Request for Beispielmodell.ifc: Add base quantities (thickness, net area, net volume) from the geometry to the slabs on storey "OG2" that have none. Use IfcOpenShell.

First a look at what the model holds.

```python
import ifcopenshell
import ifcopenshell.util.element
import ifcopenshell.util.unit

model = ifcopenshell.open("Beispielmodell.ifc")
print(model.schema)
for unit_type in ("LENGTHUNIT", "AREAUNIT", "VOLUMEUNIT"):
    print(unit_type, ifcopenshell.util.unit.calculate_unit_scale(model, unit_type))
storey = next(s for s in model.by_type("IfcBuildingStorey") if s.Name == "OG2")
slabs = [e for e in ifcopenshell.util.element.get_decomposition(storey) if e.is_a("IfcSlab")]
for e in sorted(slabs, key=lambda e: e.id()):
    print(e.id(), e.is_a(), e.Name, list(ifcopenshell.util.element.get_psets(e, qtos_only=True)), sep=" | ")
```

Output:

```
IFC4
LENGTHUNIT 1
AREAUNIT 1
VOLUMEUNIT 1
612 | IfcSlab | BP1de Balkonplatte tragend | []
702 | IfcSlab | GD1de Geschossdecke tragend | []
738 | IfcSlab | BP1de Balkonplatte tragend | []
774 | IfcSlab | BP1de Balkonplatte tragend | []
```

```python
import ifcopenshell
import ifcopenshell.api.pset
import ifcopenshell.geom
import ifcopenshell.util.element
import ifcopenshell.util.shape
import ifcopenshell.util.unit

model = ifcopenshell.open("Beispielmodell.ifc")
unit_scale = ifcopenshell.util.unit.calculate_unit_scale(model)
area_scale = ifcopenshell.util.unit.calculate_unit_scale(model, "AREAUNIT")
volume_scale = ifcopenshell.util.unit.calculate_unit_scale(model, "VOLUMEUNIT")
settings = ifcopenshell.geom.settings()

storey = next(s for s in model.by_type("IfcBuildingStorey") if s.Name == "OG2")
slabs = [e for e in ifcopenshell.util.element.get_decomposition(storey) if e.is_a("IfcSlab")]

for e in sorted(slabs, key=lambda e: e.id()):
    if ifcopenshell.util.element.get_psets(e, qtos_only=True, should_inherit=False):
        continue
    # Geometry comes back in metres, in the element's own axes.
    shape = ifcopenshell.geom.create_shape(settings, e)
    values = {
        "Width": ifcopenshell.util.shape.get_z(shape.geometry) / unit_scale,
        "NetArea": ifcopenshell.util.shape.get_footprint_area(shape.geometry) / area_scale,
        "NetVolume": ifcopenshell.util.shape.get_volume(shape.geometry) / volume_scale,
    }
    qto = ifcopenshell.api.pset.add_qto(model, product=e, name="Qto_SlabBaseQuantities")
    ifcopenshell.api.pset.edit_qto(model, qto=qto, properties=values)
    print(e.id(), {k: round(v, 3) for k, v in values.items()})

model.write("Beispielmodell_rev.ifc")
```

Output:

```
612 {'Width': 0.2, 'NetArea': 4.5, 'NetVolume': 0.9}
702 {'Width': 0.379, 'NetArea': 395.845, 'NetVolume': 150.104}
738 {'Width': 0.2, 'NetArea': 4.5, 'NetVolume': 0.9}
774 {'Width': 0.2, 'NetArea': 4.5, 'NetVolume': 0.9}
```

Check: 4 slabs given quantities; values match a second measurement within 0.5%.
